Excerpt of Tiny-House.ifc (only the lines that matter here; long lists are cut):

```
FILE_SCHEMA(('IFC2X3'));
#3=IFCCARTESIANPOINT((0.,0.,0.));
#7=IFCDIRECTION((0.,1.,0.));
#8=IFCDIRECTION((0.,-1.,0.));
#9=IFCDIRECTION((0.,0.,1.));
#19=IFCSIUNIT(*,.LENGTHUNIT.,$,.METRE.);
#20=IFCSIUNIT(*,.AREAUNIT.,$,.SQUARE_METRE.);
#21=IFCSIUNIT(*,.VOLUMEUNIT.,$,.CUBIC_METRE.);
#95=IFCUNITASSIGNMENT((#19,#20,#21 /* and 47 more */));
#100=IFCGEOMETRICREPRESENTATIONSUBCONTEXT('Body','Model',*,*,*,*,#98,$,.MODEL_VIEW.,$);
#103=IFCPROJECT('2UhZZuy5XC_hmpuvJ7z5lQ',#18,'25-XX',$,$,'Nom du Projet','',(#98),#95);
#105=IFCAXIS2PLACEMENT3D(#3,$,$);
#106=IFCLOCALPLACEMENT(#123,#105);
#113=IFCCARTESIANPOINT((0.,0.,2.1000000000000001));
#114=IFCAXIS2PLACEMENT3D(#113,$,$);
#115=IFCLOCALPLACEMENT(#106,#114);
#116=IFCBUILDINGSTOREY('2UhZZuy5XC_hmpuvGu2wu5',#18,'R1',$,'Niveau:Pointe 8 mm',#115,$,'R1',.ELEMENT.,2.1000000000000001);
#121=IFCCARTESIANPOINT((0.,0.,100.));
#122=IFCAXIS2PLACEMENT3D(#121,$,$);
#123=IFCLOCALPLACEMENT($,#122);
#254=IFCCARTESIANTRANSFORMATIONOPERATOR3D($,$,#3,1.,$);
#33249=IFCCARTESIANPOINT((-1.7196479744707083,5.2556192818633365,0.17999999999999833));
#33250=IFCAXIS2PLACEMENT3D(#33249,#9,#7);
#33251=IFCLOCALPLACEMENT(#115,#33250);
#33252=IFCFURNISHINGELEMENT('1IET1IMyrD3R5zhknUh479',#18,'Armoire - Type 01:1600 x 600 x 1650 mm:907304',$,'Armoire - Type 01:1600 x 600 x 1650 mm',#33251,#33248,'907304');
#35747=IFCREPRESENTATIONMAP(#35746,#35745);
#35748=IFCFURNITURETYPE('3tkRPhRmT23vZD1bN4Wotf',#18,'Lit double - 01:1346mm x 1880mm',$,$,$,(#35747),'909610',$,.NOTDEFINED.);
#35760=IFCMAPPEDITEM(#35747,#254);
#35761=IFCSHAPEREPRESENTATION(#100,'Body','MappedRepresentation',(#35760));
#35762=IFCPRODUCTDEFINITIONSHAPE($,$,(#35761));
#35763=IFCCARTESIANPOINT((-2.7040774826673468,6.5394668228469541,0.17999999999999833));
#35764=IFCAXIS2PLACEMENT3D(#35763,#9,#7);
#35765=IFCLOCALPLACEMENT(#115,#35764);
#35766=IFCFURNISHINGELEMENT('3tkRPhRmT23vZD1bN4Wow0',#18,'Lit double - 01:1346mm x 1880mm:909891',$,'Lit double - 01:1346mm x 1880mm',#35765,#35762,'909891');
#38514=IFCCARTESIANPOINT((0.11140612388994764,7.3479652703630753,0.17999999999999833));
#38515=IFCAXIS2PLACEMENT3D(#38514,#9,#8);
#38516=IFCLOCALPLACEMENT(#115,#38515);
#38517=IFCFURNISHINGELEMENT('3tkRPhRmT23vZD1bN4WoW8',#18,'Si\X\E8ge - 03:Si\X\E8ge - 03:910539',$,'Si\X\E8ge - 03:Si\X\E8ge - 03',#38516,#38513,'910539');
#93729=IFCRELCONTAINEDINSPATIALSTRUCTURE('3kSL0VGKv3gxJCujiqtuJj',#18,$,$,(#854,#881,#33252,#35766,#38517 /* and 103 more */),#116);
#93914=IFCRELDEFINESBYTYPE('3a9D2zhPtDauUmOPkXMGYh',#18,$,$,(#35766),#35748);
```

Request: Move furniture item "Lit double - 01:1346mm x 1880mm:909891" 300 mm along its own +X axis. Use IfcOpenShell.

```python
import ifcopenshell
import ifcopenshell.api.geometry
import ifcopenshell.util.placement
import ifcopenshell.util.unit

model = ifcopenshell.open("Tiny-House.ifc")
unit_scale = ifcopenshell.util.unit.calculate_unit_scale(model)

item = model.by_id(35766)
matrix = ifcopenshell.util.placement.get_local_placement(item.ObjectPlacement)
matrix[:3, 3] += matrix[:3, 0] * 0.3 / unit_scale
ifcopenshell.api.geometry.edit_object_placement(model, product=item, matrix=matrix, is_si=False)

print(ifcopenshell.util.placement.get_local_placement(item.ObjectPlacement).round(3) + 0.0)

model.write("Tiny-House_edited.ifc")
```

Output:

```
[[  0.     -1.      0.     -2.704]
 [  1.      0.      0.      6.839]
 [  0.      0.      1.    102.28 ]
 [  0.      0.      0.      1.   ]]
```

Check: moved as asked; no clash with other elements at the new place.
